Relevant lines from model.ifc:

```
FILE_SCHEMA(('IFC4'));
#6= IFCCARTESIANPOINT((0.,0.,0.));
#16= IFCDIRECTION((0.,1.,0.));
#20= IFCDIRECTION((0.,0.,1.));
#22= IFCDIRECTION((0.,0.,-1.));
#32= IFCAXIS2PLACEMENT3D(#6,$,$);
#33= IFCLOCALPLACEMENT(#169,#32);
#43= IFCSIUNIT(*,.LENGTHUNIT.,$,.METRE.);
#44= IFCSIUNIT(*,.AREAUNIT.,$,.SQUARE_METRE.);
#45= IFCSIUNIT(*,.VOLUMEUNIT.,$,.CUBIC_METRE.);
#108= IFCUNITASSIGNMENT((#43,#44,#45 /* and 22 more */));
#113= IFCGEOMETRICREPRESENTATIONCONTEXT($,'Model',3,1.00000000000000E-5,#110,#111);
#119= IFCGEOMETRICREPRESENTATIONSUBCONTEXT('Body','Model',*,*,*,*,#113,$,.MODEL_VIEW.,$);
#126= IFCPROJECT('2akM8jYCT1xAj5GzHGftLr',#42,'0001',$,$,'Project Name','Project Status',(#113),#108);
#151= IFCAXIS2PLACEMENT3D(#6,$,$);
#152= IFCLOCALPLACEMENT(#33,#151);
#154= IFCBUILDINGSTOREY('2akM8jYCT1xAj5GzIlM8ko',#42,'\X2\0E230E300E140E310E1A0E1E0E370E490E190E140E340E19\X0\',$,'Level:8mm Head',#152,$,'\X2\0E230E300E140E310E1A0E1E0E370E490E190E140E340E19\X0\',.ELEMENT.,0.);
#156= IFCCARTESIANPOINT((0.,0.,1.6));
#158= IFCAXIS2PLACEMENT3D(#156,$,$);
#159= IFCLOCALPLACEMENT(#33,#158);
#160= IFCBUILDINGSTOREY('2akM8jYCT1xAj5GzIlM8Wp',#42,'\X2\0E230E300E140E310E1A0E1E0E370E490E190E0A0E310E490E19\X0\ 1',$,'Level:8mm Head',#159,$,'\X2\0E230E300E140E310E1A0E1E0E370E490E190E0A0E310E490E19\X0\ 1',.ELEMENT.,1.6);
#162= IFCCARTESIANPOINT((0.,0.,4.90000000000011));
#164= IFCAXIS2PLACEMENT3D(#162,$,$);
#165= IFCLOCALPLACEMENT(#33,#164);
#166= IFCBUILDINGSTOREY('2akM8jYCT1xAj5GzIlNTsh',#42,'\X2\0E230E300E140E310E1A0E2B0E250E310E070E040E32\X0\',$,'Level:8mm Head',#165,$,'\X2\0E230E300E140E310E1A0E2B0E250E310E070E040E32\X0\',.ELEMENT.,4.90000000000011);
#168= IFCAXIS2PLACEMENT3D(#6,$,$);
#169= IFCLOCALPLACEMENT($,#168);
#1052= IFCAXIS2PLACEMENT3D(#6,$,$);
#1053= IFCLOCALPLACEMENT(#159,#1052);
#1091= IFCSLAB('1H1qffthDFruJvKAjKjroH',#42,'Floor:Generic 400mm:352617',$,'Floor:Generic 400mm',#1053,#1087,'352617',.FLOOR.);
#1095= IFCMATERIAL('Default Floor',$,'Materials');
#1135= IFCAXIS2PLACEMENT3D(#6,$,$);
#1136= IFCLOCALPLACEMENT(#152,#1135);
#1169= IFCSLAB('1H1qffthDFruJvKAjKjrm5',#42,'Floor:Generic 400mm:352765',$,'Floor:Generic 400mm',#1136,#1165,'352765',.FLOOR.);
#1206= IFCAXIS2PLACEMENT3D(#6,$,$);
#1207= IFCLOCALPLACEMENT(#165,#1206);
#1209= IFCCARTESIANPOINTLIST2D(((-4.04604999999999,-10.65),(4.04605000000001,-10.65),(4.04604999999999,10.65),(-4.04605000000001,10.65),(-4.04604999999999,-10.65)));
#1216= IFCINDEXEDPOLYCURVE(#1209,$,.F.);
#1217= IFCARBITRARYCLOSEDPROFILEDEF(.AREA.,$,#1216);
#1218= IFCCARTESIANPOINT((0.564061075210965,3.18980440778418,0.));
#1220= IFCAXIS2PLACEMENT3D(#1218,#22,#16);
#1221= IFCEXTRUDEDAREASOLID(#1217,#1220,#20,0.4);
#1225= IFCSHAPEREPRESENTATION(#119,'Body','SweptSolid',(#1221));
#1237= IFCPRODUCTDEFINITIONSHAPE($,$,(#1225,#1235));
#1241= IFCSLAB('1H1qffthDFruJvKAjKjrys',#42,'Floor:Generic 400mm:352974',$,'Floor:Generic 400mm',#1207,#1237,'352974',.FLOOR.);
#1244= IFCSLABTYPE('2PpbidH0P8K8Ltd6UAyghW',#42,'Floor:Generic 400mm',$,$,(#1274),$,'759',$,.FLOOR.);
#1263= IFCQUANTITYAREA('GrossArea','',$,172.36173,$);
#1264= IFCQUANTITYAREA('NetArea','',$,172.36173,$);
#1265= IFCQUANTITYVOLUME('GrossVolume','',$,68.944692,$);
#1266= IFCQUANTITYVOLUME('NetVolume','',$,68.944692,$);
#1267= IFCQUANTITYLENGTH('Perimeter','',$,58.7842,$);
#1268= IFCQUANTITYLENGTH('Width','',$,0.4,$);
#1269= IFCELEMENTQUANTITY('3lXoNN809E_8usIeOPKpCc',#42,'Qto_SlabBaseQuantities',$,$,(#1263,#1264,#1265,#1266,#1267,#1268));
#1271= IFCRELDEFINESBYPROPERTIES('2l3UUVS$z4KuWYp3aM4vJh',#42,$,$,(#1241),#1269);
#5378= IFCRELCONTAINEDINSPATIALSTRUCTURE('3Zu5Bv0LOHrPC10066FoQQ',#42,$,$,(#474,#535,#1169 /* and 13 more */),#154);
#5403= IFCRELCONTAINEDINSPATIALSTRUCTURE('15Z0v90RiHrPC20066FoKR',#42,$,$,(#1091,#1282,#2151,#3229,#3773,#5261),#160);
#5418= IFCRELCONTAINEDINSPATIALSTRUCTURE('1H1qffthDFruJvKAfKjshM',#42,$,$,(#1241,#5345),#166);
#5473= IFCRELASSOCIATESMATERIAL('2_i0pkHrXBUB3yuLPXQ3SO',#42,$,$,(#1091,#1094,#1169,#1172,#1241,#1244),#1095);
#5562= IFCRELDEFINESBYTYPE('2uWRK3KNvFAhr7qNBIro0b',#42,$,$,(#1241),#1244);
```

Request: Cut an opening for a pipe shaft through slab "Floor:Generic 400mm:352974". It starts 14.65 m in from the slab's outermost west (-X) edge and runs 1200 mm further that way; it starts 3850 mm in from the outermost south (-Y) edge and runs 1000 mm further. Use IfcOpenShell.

```python
import numpy as np
import ifcopenshell
import ifcopenshell.api.feature
import ifcopenshell.api.geometry
import ifcopenshell.api.pset
import ifcopenshell.api.root
import ifcopenshell.geom
import ifcopenshell.util.element
import ifcopenshell.util.placement
import ifcopenshell.util.representation
import ifcopenshell.util.shape
import ifcopenshell.util.unit

model = ifcopenshell.open("model.ifc")
unit_scale = ifcopenshell.util.unit.calculate_unit_scale(model)
area_scale = ifcopenshell.util.unit.calculate_unit_scale(model, "AREAUNIT")
volume_scale = ifcopenshell.util.unit.calculate_unit_scale(model, "VOLUMEUNIT")
settings = ifcopenshell.geom.settings()


def volume(element):
    """Net volume in cubic metres, openings subtracted."""
    shape = ifcopenshell.geom.create_shape(settings, element)
    return ifcopenshell.util.shape.get_volume(shape.geometry)


slab = model.by_guid("1H1qffthDFruJvKAjKjrys")
before = volume(slab)

# Extent in the slab's own axes, in metres. The edges named are its -X and -Y sides.
slab_shape = ifcopenshell.geom.create_shape(settings, slab)
vertices = ifcopenshell.util.shape.get_vertices(slab_shape.geometry)
x_min, y_min, bottom = vertices.min(axis=0)
top = vertices[:, 2].max()

opening = ifcopenshell.api.root.create_entity(model, ifc_class="IfcOpeningElement", name="Pipe shaft opening", predefined_type="OPENING")
context = ifcopenshell.util.representation.get_context(model, "Model", "Body", "MODEL_VIEW")
width, depth = 1.2, 1
outline = [(0.0, 0.0), (width, 0.0), (width, depth), (0.0, depth), (0.0, 0.0)]
# Overshoot both faces by 50 mm so the cut is clean.
shape = ifcopenshell.api.geometry.add_slab_representation(
    model, context=context, depth=top - bottom + 0.1, polyline=outline
)
ifcopenshell.api.geometry.assign_representation(model, product=opening, representation=shape)

matrix = ifcopenshell.util.placement.get_local_placement(slab.ObjectPlacement)
matrix[:, 3] = matrix @ np.append(np.array([x_min + 14.65, y_min + 3.85, bottom - 0.05]) / unit_scale, 1.0)
ifcopenshell.api.geometry.edit_object_placement(model, product=opening, matrix=matrix, is_si=False)
ifcopenshell.api.feature.add_feature(model, feature=opening, element=slab)

after = volume(slab)

# Update the slab's stored quantities.
qto = model.by_id(ifcopenshell.util.element.get_pset(slab, "Qto_SlabBaseQuantities", should_inherit=False)["id"])
ifcopenshell.api.pset.edit_qto(model, qto=qto, properties={
    "NetArea": after / (top - bottom) / area_scale,
    "NetVolume": after / volume_scale,
})

print(f"slab volume {before:.3f} -> {after:.3f} m3")

model.write("model_v2.ifc")
```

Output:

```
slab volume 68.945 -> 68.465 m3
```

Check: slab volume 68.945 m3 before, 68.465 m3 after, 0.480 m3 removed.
